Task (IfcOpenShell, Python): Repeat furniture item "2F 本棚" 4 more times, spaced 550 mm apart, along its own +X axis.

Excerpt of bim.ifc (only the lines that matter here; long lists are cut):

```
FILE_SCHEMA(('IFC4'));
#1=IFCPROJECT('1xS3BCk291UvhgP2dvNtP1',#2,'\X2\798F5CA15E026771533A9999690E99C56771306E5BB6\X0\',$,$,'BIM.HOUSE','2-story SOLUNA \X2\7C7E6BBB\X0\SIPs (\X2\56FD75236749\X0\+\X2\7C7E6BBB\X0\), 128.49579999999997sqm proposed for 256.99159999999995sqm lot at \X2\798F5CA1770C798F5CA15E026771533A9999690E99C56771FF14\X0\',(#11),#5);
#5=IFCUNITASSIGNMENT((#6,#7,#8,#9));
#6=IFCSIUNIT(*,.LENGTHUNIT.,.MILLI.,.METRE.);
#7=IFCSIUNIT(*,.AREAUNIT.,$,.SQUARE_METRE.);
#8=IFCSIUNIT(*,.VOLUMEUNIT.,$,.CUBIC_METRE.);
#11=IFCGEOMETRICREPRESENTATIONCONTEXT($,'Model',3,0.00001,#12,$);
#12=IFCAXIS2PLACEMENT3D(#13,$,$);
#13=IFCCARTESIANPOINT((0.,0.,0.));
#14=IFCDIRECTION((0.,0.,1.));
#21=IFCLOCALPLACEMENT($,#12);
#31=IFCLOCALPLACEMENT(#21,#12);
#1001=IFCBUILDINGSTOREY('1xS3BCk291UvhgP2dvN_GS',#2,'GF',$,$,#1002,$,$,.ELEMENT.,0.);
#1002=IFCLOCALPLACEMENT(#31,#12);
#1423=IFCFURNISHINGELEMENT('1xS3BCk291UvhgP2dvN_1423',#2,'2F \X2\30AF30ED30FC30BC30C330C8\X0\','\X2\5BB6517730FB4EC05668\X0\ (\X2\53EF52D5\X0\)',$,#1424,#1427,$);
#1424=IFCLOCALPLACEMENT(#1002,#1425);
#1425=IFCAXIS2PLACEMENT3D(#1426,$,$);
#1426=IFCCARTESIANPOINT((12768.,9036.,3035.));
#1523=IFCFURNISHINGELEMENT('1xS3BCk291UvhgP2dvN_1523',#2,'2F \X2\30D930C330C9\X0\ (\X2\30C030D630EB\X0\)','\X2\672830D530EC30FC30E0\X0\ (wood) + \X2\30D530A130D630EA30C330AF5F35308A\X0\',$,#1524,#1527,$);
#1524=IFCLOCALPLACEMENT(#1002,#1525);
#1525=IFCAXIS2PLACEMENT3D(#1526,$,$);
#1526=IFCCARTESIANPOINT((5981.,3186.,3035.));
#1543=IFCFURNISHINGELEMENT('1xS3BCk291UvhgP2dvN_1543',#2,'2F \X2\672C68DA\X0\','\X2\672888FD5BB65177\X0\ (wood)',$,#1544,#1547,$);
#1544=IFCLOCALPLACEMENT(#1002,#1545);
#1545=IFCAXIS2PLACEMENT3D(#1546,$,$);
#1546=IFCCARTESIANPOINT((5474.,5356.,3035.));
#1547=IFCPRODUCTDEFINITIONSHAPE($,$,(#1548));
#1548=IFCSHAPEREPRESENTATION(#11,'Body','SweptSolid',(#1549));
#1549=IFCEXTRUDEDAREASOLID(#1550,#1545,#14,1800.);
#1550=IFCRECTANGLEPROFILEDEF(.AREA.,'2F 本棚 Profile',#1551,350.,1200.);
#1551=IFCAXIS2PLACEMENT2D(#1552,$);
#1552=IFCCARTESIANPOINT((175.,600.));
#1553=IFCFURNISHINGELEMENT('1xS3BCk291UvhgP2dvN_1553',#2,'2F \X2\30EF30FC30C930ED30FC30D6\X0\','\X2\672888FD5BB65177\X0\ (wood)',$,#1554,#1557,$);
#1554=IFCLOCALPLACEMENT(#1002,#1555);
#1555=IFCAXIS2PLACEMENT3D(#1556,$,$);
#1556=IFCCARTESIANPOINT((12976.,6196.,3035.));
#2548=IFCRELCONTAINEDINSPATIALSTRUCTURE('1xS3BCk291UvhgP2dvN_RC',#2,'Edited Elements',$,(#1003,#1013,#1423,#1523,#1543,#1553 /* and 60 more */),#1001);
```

```python
import ifcopenshell
import ifcopenshell.api.geometry
import ifcopenshell.api.root
import ifcopenshell.util.element
import ifcopenshell.util.placement

model = ifcopenshell.open("bim.ifc")


def reuse_history(source, copy):
    """copy_class also copies each property set's owner history, people and application; keep the originals."""
    for rel in copy.IsDefinedBy:
        if rel.is_a("IfcRelDefinesByProperties") and (history := rel.RelatingPropertyDefinition.OwnerHistory):
            rel.RelatingPropertyDefinition.OwnerHistory = source.OwnerHistory
            ifcopenshell.util.element.remove_deep2(model, history)


source = model.by_id(1543)
base = ifcopenshell.util.placement.get_local_placement(source.ObjectPlacement)
step = base[:3, 0] * 550.0

for i in range(1, 5):
    copy = ifcopenshell.api.root.copy_class(model, product=source)
    copy.Representation = ifcopenshell.util.element.copy_deep(
        model, source.Representation, exclude=["IfcGeometricRepresentationContext", "IfcRepresentationMap"]
    )
    reuse_history(source, copy)
    matrix = base.copy()
    matrix[:3, 3] += i * step
    print("added at", matrix[:3, 3].round(3) + 0.0)
    ifcopenshell.api.geometry.edit_object_placement(model, product=copy, matrix=matrix, is_si=False)

model.write("bim_edited.ifc")
```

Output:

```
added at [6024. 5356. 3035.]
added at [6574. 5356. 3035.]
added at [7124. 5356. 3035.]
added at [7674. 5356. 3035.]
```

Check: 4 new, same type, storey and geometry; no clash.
